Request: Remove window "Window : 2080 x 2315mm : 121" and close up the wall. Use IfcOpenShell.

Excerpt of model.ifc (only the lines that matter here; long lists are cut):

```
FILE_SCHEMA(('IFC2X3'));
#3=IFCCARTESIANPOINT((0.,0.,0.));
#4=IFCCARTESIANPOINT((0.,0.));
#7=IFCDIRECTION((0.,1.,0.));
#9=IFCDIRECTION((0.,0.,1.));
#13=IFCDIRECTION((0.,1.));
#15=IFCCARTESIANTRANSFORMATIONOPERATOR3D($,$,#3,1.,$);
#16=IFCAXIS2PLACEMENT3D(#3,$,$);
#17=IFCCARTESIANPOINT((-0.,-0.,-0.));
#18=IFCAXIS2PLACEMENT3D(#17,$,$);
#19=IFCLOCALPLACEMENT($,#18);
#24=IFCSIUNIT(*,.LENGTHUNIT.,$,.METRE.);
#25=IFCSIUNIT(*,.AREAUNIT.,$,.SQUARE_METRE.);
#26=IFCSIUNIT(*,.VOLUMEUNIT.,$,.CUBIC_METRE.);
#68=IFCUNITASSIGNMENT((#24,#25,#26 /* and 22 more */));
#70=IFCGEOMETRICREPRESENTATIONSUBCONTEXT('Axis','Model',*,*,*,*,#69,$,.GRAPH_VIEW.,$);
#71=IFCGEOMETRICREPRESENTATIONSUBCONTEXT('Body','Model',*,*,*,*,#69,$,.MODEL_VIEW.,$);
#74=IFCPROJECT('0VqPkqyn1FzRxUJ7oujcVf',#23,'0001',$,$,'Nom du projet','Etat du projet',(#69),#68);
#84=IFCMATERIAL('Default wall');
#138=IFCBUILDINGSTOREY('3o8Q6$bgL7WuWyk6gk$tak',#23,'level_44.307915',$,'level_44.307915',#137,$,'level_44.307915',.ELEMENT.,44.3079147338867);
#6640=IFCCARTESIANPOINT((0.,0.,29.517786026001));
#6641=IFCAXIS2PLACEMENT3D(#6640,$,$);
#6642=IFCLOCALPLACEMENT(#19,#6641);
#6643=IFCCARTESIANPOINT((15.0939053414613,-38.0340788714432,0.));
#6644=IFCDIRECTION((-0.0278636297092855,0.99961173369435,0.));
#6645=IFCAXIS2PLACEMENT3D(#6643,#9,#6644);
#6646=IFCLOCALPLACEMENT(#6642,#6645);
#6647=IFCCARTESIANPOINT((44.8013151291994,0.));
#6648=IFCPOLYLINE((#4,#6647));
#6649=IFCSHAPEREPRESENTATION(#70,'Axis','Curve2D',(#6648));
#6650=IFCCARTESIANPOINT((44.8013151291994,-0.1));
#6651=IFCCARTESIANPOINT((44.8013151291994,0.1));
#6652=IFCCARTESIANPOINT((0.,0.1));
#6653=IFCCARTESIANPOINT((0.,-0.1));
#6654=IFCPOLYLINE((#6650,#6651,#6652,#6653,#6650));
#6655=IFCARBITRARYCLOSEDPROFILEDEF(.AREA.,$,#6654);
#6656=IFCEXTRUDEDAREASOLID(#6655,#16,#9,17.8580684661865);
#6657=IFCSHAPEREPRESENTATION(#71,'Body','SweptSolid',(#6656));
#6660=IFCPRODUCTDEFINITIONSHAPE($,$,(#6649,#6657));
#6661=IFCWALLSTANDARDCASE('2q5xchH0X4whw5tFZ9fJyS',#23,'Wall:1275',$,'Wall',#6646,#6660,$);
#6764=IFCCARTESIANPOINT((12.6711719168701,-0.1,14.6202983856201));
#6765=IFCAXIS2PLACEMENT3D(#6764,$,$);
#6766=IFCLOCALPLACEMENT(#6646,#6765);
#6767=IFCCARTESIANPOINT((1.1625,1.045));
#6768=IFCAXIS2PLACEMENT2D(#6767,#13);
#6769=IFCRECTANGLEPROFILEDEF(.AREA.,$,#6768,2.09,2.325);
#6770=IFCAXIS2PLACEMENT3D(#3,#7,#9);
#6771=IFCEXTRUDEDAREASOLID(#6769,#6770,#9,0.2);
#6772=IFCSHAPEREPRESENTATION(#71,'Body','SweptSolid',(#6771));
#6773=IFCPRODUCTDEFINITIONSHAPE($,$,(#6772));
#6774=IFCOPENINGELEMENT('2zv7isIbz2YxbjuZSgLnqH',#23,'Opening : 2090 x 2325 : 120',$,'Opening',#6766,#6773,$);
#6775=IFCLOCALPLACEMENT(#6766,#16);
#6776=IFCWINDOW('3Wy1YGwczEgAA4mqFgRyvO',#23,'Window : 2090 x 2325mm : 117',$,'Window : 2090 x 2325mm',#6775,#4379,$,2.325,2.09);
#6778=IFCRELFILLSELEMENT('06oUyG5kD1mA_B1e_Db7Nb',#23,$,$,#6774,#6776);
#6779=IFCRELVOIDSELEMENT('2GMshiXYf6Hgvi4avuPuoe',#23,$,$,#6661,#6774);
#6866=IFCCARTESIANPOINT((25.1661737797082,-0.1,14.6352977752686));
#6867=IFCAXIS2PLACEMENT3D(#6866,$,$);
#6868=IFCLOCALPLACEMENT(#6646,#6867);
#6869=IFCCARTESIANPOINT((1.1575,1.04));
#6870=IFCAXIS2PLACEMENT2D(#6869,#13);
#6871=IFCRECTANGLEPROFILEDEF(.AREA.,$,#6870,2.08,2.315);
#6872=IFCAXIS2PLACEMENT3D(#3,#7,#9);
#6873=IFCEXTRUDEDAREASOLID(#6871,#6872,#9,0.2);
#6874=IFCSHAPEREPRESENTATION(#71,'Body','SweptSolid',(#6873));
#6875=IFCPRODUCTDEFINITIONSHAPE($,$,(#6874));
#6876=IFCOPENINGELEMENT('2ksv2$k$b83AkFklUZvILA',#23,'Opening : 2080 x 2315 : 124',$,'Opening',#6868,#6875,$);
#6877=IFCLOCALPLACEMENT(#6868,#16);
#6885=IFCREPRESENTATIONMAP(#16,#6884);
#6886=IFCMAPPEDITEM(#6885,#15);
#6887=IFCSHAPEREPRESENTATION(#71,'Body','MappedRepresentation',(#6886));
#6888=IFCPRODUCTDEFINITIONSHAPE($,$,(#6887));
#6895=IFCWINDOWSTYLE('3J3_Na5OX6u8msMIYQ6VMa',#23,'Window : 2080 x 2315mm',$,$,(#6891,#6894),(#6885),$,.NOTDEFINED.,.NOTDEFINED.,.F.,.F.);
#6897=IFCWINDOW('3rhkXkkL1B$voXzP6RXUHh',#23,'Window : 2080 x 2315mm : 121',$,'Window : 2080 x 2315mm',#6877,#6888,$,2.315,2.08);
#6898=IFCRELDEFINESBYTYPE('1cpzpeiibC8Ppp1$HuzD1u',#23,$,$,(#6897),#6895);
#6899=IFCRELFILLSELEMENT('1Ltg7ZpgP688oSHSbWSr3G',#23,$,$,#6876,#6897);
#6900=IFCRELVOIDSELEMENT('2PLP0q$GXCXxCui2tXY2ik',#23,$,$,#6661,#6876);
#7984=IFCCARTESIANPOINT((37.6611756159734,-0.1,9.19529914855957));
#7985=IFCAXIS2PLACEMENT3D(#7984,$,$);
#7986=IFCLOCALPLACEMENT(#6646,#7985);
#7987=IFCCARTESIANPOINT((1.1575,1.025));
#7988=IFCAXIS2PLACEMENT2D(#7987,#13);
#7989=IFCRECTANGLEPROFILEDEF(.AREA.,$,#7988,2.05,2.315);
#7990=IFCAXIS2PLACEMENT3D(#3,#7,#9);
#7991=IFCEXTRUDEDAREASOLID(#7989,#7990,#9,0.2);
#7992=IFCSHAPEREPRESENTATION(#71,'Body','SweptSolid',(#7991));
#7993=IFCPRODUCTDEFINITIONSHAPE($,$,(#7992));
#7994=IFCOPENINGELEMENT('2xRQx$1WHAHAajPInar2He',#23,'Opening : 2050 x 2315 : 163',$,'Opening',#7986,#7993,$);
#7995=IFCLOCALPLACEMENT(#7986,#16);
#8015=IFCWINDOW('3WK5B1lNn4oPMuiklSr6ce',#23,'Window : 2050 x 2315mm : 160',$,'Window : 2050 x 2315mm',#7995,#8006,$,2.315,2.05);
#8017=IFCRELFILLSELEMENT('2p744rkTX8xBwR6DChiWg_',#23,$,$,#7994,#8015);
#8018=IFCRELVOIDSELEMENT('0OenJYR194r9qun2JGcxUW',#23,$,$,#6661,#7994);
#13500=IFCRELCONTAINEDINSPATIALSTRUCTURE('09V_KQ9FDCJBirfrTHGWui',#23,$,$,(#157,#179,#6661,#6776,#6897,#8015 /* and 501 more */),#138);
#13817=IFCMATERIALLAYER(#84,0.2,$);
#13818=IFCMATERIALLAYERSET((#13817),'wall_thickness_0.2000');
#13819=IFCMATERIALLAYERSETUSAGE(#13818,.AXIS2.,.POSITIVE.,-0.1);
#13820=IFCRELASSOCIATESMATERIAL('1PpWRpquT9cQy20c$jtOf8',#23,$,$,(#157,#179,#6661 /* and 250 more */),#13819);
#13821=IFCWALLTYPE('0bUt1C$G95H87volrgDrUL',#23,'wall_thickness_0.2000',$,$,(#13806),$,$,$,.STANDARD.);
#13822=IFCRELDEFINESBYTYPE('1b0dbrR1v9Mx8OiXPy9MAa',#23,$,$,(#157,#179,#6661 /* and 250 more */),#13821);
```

```python
import ifcopenshell
import ifcopenshell.api.feature
import ifcopenshell.api.root
import ifcopenshell.geom
import ifcopenshell.util.shape

model = ifcopenshell.open("model.ifc")
settings = ifcopenshell.geom.settings()


def volume(element):
    """Net volume in cubic metres, openings subtracted."""
    shape = ifcopenshell.geom.create_shape(settings, element)
    return ifcopenshell.util.shape.get_volume(shape.geometry)


window = model.by_id(6897)
opening = window.FillsVoids[0].RelatingOpeningElement
wall = opening.VoidsElements[0].RelatingBuildingElement
before = volume(wall)

ifcopenshell.api.root.remove_product(model, product=window)
ifcopenshell.api.feature.remove_feature(model, feature=opening)

after = volume(wall)

print(f"wall volume {before:.3f} -> {after:.3f} m3")

model.write("model_v2.ifc")
```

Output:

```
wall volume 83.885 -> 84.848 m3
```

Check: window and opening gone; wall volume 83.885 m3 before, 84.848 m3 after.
